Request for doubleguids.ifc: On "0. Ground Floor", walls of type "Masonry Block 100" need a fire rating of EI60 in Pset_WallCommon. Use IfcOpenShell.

First a look at what the model holds.

```python
import ifcopenshell
import ifcopenshell.util.element

model = ifcopenshell.open("doubleguids.ifc")
print(model.schema)
storey = next(s for s in model.by_type("IfcBuildingStorey") if s.Name == "0. Ground Floor")
walls = [e for e in ifcopenshell.util.element.get_decomposition(storey) if e.is_a("IfcWall")]
seen = {}
for e in walls:
    element_type = ifcopenshell.util.element.get_type(e)
    key = (element_type.Name if element_type != e and element_type else None, ifcopenshell.util.element.get_pset(e, "Pset_WallCommon", "FireRating"))
    seen[key] = seen.get(key, 0) + 1
for (name, value), count in sorted(seen.items(), key=str):
    print(count, "x", name, "|", value)
```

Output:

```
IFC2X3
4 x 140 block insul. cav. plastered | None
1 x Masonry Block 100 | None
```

```python
import ifcopenshell
import ifcopenshell.api.pset
import ifcopenshell.util.element

model = ifcopenshell.open("doubleguids.ifc")

storey = next(s for s in model.by_type("IfcBuildingStorey") if s.Name == "0. Ground Floor")
walls = [e for e in ifcopenshell.util.element.get_decomposition(storey) if e.is_a("IfcWall")]

count = 0
for e in walls:
    element_type = ifcopenshell.util.element.get_type(e)
    if element_type in (None, e) or element_type.Name != "Masonry Block 100":
        continue
    # add_pset returns the element's existing set when there is one.
    pset = ifcopenshell.api.pset.add_pset(model, product=e, name="Pset_WallCommon")
    ifcopenshell.api.pset.edit_pset(model, pset=pset, properties={"FireRating": "EI60"})
    count += 1

print(count, "walls updated")

model.write("doubleguids_edited.ifc")
```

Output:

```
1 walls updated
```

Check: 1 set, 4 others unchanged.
